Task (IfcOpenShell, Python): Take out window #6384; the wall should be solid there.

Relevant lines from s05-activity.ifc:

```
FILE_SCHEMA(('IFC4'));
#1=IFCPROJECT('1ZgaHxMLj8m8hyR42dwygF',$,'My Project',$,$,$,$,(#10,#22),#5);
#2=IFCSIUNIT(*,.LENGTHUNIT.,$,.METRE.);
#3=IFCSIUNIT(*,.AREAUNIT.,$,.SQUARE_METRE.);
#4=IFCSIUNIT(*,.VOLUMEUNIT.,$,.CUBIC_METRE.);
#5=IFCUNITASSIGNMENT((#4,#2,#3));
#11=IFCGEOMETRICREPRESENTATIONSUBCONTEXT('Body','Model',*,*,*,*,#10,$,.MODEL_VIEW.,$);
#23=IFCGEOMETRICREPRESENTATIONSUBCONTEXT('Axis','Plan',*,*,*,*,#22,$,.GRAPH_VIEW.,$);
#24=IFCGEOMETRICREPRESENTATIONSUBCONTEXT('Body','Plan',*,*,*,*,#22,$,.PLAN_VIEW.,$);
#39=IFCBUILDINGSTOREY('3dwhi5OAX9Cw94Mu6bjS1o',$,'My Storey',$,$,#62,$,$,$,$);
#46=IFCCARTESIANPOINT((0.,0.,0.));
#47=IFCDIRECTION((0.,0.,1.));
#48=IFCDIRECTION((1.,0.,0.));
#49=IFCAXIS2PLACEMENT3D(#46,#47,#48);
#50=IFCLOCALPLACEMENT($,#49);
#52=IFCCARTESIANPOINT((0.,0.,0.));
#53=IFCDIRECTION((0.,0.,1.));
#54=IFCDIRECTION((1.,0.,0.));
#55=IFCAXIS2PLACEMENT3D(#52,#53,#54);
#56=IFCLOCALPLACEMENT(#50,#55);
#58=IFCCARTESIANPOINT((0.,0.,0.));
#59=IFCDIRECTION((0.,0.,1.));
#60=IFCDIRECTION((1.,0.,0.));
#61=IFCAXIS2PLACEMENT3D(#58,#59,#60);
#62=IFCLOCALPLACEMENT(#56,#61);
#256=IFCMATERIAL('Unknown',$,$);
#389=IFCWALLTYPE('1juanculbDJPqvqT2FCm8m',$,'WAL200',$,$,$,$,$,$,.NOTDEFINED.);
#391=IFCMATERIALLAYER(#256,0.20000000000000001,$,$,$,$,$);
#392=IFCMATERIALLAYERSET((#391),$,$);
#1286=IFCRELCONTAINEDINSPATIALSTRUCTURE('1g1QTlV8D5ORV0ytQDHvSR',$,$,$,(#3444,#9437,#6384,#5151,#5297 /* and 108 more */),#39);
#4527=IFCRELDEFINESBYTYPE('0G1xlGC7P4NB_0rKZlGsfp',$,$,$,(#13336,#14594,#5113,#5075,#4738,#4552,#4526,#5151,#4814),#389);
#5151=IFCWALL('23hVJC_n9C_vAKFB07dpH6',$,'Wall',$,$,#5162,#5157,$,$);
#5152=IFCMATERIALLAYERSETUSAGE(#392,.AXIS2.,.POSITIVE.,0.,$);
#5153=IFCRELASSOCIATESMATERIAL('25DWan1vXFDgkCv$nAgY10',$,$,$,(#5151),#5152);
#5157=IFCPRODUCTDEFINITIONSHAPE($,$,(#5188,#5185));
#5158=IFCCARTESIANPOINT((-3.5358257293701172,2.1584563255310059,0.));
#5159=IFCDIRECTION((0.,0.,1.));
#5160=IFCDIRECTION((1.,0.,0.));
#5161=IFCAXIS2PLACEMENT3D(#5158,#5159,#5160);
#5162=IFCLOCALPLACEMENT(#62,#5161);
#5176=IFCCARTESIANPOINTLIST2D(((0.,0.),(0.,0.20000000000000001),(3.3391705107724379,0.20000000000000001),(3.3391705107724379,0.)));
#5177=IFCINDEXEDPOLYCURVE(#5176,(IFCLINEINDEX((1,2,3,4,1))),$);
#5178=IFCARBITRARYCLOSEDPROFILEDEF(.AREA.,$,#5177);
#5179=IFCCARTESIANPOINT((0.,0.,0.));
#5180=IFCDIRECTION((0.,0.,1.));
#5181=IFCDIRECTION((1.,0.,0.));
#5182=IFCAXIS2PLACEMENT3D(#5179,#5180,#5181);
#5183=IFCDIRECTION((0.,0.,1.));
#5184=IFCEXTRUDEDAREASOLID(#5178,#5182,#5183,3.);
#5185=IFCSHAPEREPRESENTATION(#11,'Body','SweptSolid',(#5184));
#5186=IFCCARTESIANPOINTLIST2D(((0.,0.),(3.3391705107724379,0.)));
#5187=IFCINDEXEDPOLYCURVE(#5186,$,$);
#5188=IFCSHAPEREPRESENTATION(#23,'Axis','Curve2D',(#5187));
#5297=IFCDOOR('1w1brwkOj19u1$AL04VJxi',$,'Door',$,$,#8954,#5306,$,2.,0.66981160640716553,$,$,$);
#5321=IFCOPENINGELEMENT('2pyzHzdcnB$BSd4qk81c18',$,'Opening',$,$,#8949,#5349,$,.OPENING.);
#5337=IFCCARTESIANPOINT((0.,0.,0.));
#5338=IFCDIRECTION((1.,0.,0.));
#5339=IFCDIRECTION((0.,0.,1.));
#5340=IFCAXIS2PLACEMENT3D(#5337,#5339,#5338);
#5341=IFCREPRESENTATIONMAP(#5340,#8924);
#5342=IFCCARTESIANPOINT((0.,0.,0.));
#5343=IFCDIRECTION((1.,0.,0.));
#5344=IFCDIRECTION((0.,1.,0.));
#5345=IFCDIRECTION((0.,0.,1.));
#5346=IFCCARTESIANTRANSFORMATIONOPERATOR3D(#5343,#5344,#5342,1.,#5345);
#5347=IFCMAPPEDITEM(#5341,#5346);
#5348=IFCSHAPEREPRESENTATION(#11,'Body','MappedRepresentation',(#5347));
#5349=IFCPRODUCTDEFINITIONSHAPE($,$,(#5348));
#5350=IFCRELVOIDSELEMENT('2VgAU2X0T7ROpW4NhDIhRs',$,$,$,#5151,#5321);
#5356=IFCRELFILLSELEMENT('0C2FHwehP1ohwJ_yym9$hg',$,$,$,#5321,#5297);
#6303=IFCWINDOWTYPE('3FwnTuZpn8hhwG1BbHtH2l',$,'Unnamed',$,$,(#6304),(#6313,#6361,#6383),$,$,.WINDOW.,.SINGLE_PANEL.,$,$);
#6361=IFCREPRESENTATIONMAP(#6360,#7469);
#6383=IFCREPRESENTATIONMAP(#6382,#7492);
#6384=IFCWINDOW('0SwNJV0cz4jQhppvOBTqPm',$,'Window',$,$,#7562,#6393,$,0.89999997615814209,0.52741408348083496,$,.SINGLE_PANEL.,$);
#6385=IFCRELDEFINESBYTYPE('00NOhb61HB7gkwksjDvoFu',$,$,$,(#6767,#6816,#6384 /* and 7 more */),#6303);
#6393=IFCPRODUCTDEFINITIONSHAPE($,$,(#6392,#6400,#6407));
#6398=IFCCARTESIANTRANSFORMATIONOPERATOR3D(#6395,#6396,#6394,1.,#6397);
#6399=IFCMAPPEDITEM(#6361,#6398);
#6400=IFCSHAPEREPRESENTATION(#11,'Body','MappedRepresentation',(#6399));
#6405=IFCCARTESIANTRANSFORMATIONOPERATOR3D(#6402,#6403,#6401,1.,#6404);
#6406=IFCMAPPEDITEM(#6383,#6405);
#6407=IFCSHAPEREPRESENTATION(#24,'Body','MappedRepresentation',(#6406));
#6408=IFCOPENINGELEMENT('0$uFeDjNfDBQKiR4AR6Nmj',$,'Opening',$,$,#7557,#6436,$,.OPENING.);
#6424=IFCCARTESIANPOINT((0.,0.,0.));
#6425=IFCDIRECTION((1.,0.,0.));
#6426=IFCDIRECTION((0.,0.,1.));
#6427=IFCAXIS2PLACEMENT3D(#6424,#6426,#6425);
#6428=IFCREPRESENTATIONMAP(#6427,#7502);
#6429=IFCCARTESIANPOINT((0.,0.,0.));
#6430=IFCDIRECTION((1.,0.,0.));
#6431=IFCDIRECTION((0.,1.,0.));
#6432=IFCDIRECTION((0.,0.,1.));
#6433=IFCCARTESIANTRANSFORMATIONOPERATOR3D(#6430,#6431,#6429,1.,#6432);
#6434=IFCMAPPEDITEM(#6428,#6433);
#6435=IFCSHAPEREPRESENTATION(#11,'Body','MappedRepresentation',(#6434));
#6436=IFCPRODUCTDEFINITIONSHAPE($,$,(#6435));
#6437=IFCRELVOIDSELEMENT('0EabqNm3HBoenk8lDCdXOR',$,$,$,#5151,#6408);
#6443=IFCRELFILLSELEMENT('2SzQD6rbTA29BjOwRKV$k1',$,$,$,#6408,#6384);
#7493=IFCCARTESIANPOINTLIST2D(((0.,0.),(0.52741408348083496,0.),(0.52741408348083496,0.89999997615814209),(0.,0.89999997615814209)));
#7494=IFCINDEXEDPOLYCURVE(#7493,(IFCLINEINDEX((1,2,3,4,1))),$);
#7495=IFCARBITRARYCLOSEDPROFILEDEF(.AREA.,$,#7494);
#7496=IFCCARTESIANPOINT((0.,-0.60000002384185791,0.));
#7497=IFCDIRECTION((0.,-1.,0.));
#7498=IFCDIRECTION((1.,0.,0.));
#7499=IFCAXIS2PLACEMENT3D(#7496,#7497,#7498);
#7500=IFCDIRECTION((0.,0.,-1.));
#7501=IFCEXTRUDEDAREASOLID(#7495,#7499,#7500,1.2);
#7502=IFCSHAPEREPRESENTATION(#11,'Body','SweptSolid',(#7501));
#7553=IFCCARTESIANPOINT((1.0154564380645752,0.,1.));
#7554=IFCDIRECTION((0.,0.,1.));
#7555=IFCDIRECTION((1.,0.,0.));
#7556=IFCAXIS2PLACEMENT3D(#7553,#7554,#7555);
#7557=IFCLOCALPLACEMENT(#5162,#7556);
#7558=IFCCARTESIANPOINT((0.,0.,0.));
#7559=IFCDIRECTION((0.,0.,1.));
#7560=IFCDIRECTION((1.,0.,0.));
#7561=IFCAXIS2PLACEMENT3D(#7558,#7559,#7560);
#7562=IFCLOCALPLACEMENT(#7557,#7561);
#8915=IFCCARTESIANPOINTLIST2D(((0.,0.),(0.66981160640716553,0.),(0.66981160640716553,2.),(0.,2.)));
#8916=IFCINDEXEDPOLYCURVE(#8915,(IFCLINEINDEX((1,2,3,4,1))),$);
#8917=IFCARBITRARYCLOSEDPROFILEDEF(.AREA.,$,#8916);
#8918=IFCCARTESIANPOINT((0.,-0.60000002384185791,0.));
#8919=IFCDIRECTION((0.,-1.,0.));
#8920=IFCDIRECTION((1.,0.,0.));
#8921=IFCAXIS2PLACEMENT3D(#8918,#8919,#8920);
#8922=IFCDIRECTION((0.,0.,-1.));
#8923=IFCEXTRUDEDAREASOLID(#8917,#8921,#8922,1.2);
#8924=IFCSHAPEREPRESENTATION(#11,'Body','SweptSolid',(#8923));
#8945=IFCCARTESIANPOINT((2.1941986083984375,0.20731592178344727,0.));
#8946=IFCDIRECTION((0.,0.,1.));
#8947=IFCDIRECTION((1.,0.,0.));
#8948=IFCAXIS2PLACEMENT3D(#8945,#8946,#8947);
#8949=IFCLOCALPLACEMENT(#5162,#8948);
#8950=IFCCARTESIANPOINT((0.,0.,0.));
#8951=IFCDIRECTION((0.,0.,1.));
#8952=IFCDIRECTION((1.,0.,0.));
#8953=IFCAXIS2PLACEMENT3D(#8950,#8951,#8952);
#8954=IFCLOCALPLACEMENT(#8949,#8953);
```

```python
import ifcopenshell
import ifcopenshell.api.feature
import ifcopenshell.api.root
import ifcopenshell.geom
import ifcopenshell.util.shape

model = ifcopenshell.open("s05-activity.ifc")
settings = ifcopenshell.geom.settings()


def volume(element):
    """Net volume in cubic metres, openings subtracted."""
    shape = ifcopenshell.geom.create_shape(settings, element)
    return ifcopenshell.util.shape.get_volume(shape.geometry)


window = model.by_guid("0SwNJV0cz4jQhppvOBTqPm")
opening = window.FillsVoids[0].RelatingOpeningElement
wall = opening.VoidsElements[0].RelatingBuildingElement
before = volume(wall)

ifcopenshell.api.root.remove_product(model, product=window)
ifcopenshell.api.feature.remove_feature(model, feature=opening)

after = volume(wall)

print(f"wall volume {before:.3f} -> {after:.3f} m3")

model.write("s05-activity_rev.ifc")
```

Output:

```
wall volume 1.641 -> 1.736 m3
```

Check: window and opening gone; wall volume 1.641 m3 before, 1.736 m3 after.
